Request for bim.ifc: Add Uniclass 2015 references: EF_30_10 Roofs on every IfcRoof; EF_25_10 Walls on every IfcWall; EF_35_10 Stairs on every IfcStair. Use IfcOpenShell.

First a look at what the model holds.

```python
import ifcopenshell

model = ifcopenshell.open("bim.ifc")
print(model.schema)
print("classifications:", [c.Name for c in model.by_type("IfcClassification")])
for ifc_class in ("IfcDoor", "IfcRoof", "IfcStair", "IfcWall", "IfcWindow"):
    print(ifc_class, len(model.by_type(ifc_class)))
```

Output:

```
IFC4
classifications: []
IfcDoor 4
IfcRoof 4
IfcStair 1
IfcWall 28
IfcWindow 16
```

```python
import ifcopenshell
import ifcopenshell.api.classification

model = ifcopenshell.open("bim.ifc")

system = ifcopenshell.api.classification.add_classification(model, classification="Uniclass 2015")

codes = {
    "IfcRoof": ("EF_30_10", "Roofs"),
    "IfcWall": ("EF_25_10", "Walls"),
    "IfcStair": ("EF_35_10", "Stairs"),
}
for ifc_class, (code, name) in codes.items():
    products = model.by_type(ifc_class)
    ifcopenshell.api.classification.add_reference(
        model, products=products, classification=system, identification=code, name=name
    )
    print(code, len(products))

model.write("bim_updated.ifc")
```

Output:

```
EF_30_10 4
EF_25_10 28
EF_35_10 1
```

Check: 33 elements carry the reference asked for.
